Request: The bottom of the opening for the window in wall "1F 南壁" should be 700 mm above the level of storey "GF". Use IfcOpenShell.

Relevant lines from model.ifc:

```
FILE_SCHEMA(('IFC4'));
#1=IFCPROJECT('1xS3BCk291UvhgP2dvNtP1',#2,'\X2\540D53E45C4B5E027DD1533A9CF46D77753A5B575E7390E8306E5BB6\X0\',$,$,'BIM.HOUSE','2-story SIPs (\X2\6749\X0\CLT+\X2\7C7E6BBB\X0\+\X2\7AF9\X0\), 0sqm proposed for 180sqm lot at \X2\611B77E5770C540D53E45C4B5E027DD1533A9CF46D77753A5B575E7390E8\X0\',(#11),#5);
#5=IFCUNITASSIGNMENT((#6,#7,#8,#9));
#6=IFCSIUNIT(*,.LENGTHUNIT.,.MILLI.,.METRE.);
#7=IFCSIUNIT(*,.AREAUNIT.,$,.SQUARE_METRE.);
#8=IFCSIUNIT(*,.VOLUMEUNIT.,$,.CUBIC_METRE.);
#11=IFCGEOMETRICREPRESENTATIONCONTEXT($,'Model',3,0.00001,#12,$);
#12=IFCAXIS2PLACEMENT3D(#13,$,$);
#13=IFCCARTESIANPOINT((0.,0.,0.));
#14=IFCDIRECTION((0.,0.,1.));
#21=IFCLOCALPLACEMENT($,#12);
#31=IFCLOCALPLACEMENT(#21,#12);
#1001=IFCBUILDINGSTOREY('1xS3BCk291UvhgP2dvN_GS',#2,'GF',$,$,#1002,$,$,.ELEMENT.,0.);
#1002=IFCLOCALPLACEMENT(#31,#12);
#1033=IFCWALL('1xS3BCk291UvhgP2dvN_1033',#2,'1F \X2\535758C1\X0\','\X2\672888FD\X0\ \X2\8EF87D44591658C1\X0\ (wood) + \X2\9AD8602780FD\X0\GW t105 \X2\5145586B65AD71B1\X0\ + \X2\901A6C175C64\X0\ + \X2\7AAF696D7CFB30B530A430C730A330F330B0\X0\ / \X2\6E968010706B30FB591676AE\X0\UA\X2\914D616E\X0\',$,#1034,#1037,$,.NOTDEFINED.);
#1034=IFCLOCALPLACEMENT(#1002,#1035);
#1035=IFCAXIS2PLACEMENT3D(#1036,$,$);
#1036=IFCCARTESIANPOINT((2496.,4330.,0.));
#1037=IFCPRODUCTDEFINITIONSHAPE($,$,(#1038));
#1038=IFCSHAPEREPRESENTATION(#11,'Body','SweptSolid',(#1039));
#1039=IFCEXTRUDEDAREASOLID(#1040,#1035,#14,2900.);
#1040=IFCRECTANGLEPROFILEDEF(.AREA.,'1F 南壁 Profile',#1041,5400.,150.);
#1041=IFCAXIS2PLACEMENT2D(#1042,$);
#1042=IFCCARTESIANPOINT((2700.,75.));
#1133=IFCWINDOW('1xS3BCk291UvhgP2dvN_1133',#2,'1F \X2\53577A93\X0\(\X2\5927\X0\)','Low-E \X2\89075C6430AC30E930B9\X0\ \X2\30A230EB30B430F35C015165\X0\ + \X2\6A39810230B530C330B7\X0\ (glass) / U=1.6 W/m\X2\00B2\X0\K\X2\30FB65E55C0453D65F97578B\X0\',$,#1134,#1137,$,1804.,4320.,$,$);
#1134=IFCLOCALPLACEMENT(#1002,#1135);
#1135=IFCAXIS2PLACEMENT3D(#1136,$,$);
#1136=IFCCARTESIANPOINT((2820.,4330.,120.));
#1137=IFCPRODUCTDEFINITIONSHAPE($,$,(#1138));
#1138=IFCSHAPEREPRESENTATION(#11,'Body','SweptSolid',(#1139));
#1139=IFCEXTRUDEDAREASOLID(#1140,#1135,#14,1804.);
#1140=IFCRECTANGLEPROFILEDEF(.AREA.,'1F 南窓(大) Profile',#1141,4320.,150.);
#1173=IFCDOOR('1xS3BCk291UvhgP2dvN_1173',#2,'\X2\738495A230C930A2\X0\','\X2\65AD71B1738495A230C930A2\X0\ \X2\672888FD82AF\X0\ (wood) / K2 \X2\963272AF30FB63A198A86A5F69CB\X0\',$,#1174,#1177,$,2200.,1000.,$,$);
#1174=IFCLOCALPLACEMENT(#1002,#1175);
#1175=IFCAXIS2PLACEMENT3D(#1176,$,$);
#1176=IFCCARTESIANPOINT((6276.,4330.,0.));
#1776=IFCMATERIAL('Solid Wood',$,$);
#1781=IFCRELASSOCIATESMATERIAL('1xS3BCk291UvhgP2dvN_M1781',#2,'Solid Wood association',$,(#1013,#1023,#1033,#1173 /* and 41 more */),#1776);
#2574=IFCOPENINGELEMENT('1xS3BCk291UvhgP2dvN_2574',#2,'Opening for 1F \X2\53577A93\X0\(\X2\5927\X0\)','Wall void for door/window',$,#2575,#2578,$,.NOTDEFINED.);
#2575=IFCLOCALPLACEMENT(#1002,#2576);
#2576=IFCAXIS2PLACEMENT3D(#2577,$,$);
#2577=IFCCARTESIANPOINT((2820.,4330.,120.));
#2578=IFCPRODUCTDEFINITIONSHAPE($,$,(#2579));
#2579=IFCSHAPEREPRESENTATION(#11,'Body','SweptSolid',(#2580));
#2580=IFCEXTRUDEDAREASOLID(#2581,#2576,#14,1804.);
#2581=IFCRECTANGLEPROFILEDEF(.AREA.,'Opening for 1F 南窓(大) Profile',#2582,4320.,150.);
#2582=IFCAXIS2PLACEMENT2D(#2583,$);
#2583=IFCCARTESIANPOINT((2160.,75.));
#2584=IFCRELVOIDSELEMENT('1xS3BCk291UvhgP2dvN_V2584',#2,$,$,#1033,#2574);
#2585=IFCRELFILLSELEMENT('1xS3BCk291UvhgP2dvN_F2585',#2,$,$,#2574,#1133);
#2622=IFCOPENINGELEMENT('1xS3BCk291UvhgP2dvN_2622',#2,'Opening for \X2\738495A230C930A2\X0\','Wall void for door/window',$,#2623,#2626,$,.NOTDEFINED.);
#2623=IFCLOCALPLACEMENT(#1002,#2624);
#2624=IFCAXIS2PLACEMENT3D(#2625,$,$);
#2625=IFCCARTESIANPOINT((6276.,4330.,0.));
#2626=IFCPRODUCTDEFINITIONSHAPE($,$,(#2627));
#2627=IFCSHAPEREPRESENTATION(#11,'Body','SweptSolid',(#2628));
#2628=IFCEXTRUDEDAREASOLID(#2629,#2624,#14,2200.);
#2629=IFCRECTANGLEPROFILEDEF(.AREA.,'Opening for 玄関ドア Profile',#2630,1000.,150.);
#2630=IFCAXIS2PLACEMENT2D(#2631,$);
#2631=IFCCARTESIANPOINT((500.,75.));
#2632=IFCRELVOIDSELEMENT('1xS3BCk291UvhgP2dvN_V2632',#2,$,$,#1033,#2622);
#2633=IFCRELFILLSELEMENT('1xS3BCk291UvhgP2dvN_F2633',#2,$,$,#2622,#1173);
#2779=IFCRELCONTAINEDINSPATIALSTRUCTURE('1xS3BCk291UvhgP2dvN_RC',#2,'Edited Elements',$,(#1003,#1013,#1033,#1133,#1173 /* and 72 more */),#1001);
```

```python
import numpy as np
import ifcopenshell
import ifcopenshell.api.geometry
import ifcopenshell.geom
import ifcopenshell.util.element
import ifcopenshell.util.placement
import ifcopenshell.util.shape
import ifcopenshell.util.unit

model = ifcopenshell.open("model.ifc")
unit_scale = ifcopenshell.util.unit.calculate_unit_scale(model)

window = model.by_guid("1xS3BCk291UvhgP2dvN_1133")
opening = window.FillsVoids[0].RelatingOpeningElement
storey = ifcopenshell.util.element.get_container(window, ifc_class="IfcBuildingStorey")
level = ifcopenshell.util.placement.get_local_placement(storey.ObjectPlacement)[2, 3]

# The opening's origin need not be at the sill, so measure its lowest point.
shape = ifcopenshell.geom.create_shape(ifcopenshell.geom.settings(), opening)
bottom = ifcopenshell.util.shape.get_shape_bottom_elevation(shape, shape.geometry) / unit_scale
dz = level + 0.7 / unit_scale - bottom

shift = np.array([0.0, 0.0, dz])
# The window is not placed relative to its opening, so move both.
for product in (opening, window):
    matrix = ifcopenshell.util.placement.get_local_placement(product.ObjectPlacement)
    matrix[:3, 3] += shift
    ifcopenshell.api.geometry.edit_object_placement(model, product=product, matrix=matrix, is_si=False)

print(f"moved by {dz * unit_scale:+.3f} m")

model.write("model_v2.ifc")
```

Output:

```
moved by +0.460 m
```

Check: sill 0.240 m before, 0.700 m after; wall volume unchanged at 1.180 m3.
